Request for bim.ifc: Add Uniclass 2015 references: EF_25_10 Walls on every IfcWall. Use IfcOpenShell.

First a look at what the model holds.

```python
import ifcopenshell

model = ifcopenshell.open("bim.ifc")
print(model.schema)
print("classifications:", [c.Name for c in model.by_type("IfcClassification")])
for ifc_class in ("IfcDoor", "IfcRoof", "IfcStair", "IfcWall", "IfcWindow"):
    print(ifc_class, len(model.by_type(ifc_class)))
```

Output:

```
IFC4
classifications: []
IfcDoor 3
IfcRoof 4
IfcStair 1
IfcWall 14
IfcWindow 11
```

```python
import ifcopenshell
import ifcopenshell.api.classification

model = ifcopenshell.open("bim.ifc")

system = ifcopenshell.api.classification.add_classification(model, classification="Uniclass 2015")

codes = {
    "IfcWall": ("EF_25_10", "Walls"),
}
for ifc_class, (code, name) in codes.items():
    products = model.by_type(ifc_class)
    ifcopenshell.api.classification.add_reference(
        model, products=products, classification=system, identification=code, name=name
    )
    print(code, len(products))

model.write("bim_edited.ifc")
```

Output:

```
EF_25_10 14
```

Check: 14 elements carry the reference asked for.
